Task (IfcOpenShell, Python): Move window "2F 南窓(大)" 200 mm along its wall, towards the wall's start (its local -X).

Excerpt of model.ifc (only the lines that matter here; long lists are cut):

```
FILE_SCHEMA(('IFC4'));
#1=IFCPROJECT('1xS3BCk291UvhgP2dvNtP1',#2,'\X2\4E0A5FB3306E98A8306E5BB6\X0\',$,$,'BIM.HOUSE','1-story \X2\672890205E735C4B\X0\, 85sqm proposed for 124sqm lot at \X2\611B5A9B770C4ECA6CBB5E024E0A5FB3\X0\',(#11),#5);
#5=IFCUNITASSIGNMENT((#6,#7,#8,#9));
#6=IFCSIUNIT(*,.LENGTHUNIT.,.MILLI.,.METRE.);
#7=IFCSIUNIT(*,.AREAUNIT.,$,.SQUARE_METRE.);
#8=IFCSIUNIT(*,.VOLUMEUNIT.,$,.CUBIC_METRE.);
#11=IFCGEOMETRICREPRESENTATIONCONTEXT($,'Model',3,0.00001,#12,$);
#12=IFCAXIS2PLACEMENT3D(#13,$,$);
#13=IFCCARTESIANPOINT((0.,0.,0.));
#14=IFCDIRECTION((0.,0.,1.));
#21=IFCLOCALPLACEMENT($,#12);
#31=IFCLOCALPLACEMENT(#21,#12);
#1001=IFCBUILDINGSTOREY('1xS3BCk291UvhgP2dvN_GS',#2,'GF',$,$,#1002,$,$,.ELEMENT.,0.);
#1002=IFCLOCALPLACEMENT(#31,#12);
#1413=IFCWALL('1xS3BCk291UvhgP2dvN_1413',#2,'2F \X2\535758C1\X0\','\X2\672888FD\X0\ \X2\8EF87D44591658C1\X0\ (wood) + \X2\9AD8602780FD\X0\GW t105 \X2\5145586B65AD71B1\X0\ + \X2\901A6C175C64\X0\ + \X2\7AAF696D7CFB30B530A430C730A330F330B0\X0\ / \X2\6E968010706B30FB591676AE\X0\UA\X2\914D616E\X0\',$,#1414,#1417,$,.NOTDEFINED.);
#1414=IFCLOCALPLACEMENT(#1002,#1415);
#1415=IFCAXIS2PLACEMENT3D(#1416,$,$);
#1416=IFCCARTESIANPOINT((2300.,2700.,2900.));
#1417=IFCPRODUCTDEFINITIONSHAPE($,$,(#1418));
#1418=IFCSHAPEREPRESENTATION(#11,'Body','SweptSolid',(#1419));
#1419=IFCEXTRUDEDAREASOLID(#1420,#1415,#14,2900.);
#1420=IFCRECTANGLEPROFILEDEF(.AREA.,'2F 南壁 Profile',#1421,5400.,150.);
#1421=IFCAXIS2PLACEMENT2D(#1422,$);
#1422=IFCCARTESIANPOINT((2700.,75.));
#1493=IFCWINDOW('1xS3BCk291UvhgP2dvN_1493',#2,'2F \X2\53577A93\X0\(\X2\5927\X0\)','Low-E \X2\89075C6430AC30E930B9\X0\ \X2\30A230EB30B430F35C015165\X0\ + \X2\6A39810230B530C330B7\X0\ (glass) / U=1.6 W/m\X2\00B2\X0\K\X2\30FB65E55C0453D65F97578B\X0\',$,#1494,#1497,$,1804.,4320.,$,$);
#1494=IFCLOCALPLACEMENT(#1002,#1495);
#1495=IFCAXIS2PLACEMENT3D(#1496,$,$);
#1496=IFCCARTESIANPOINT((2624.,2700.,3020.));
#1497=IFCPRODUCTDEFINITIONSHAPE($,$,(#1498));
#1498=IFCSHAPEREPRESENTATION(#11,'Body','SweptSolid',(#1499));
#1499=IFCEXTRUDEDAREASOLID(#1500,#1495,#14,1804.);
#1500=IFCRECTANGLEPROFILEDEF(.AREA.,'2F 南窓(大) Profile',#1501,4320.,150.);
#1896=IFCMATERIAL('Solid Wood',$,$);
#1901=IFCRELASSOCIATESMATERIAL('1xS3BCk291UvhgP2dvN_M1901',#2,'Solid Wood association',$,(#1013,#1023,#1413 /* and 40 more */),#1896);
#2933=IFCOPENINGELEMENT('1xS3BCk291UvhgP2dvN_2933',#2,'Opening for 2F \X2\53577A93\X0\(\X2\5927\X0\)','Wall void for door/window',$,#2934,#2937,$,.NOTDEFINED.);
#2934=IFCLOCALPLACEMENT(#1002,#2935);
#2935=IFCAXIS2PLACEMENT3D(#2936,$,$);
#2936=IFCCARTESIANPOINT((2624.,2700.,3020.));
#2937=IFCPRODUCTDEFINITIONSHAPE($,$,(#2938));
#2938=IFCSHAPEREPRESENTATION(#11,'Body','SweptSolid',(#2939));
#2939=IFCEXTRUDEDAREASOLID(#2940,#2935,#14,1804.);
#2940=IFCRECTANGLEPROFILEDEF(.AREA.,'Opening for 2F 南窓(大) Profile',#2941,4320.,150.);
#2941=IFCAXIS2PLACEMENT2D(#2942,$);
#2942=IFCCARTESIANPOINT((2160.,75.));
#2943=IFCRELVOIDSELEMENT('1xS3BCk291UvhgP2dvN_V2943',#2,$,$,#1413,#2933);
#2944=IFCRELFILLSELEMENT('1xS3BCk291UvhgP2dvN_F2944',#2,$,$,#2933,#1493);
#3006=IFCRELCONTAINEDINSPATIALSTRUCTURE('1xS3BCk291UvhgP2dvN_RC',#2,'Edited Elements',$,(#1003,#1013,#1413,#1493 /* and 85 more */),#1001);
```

```python
import ifcopenshell
import ifcopenshell.api.geometry
import ifcopenshell.util.placement

model = ifcopenshell.open("model.ifc")

window = model.by_id(1493)
opening = window.FillsVoids[0].RelatingOpeningElement
wall = opening.VoidsElements[0].RelatingBuildingElement

wall_matrix = ifcopenshell.util.placement.get_local_placement(wall.ObjectPlacement)
shift = wall_matrix[:3, 0] * -200.0
before = ifcopenshell.util.placement.get_local_placement(window.ObjectPlacement)[:3, 3].copy()

# The window is not placed relative to its opening, so move both.
for product in (opening, window):
    matrix = ifcopenshell.util.placement.get_local_placement(product.ObjectPlacement)
    matrix[:3, 3] += shift
    ifcopenshell.api.geometry.edit_object_placement(model, product=product, matrix=matrix, is_si=False)

after = ifcopenshell.util.placement.get_local_placement(window.ObjectPlacement)[:3, 3]
print("window moved by", (after - before).round(3) + 0.0)

model.write("model_edited.ifc")
```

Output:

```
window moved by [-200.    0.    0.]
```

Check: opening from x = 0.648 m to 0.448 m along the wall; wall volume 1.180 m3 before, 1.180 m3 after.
